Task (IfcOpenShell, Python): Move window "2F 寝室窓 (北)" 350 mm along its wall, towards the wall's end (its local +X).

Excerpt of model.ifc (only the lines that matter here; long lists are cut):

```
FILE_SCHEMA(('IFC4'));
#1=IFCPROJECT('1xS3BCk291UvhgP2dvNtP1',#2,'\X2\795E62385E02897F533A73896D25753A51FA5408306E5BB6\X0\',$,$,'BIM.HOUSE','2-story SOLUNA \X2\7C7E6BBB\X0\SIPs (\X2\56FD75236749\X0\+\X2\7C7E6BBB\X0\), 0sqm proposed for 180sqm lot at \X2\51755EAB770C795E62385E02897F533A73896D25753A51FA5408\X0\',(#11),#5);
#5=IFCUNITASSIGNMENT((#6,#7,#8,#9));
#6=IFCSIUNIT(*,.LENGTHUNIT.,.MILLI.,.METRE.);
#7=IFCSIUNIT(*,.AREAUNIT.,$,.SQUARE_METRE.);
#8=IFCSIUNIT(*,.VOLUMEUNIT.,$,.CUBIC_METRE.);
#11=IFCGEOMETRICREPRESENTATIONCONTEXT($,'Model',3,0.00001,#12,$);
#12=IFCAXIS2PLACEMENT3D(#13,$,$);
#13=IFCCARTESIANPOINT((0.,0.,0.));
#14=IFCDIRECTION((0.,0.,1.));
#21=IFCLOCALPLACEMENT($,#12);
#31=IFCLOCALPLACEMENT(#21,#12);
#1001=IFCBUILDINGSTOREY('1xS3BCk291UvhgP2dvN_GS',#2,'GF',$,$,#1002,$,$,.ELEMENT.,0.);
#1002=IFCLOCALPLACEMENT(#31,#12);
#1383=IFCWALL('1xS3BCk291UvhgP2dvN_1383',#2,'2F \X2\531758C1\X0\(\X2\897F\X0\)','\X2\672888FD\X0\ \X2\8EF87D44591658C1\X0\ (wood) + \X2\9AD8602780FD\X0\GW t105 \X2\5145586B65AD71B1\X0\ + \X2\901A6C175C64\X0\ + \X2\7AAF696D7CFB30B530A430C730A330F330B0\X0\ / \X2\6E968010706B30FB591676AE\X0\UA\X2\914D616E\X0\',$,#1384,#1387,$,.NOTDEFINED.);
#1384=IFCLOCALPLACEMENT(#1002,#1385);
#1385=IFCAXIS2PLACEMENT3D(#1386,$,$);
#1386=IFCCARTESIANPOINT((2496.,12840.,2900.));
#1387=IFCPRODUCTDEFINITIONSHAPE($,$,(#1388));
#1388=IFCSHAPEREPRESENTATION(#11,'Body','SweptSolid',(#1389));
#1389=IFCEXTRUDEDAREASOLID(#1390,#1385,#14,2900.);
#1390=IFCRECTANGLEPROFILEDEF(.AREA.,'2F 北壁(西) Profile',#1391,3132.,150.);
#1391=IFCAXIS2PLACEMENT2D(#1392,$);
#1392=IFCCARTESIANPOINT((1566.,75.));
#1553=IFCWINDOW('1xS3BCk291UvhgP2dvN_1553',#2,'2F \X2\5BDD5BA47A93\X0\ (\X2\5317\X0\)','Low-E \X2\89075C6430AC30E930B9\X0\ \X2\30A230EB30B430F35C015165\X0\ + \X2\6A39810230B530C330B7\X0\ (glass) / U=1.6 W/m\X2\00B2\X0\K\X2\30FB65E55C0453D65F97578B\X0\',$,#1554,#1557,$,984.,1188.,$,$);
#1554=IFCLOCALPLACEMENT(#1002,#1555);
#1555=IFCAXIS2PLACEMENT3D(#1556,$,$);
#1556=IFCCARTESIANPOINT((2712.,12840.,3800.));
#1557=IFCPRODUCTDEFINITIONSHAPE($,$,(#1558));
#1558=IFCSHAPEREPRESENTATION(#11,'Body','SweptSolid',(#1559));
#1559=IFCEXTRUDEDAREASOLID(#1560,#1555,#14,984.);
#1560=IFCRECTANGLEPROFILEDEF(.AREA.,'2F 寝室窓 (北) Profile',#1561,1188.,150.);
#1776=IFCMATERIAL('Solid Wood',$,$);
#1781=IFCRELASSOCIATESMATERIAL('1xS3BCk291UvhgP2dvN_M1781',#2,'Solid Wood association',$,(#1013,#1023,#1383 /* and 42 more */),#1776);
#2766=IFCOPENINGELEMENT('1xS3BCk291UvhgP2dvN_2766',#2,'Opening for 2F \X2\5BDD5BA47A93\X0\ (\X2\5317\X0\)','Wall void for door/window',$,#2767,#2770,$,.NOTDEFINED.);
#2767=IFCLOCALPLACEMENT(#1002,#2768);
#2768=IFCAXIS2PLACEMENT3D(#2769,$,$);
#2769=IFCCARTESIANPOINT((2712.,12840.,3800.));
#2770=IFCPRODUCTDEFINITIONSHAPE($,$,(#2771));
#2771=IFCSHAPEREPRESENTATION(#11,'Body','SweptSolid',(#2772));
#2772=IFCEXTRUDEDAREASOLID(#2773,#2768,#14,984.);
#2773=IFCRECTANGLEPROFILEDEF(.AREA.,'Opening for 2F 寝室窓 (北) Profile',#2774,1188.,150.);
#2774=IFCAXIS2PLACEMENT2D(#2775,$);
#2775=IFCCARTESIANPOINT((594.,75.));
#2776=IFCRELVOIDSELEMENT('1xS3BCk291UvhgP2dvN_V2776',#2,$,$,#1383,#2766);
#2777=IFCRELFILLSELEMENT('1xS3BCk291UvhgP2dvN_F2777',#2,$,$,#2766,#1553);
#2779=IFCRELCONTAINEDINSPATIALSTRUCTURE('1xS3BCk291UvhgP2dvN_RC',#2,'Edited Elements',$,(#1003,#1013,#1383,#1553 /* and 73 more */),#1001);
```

```python
import ifcopenshell
import ifcopenshell.api.geometry
import ifcopenshell.util.placement
import ifcopenshell.util.unit

model = ifcopenshell.open("model.ifc")
unit_scale = ifcopenshell.util.unit.calculate_unit_scale(model)

window = model.by_guid("1xS3BCk291UvhgP2dvN_1553")
opening = window.FillsVoids[0].RelatingOpeningElement
wall = opening.VoidsElements[0].RelatingBuildingElement

wall_matrix = ifcopenshell.util.placement.get_local_placement(wall.ObjectPlacement)
shift = wall_matrix[:3, 0] * 0.35 / unit_scale
before = ifcopenshell.util.placement.get_local_placement(window.ObjectPlacement)[:3, 3].copy()

# The window is not placed relative to its opening, so move both.
for product in (opening, window):
    matrix = ifcopenshell.util.placement.get_local_placement(product.ObjectPlacement)
    matrix[:3, 3] += shift
    ifcopenshell.api.geometry.edit_object_placement(model, product=product, matrix=matrix, is_si=False)

after = ifcopenshell.util.placement.get_local_placement(window.ObjectPlacement)[:3, 3]
print("window moved by", (after - before).round(3) + 0.0)

model.write("model-out.ifc")
```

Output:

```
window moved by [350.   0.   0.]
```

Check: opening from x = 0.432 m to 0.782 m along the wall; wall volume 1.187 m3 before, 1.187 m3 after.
